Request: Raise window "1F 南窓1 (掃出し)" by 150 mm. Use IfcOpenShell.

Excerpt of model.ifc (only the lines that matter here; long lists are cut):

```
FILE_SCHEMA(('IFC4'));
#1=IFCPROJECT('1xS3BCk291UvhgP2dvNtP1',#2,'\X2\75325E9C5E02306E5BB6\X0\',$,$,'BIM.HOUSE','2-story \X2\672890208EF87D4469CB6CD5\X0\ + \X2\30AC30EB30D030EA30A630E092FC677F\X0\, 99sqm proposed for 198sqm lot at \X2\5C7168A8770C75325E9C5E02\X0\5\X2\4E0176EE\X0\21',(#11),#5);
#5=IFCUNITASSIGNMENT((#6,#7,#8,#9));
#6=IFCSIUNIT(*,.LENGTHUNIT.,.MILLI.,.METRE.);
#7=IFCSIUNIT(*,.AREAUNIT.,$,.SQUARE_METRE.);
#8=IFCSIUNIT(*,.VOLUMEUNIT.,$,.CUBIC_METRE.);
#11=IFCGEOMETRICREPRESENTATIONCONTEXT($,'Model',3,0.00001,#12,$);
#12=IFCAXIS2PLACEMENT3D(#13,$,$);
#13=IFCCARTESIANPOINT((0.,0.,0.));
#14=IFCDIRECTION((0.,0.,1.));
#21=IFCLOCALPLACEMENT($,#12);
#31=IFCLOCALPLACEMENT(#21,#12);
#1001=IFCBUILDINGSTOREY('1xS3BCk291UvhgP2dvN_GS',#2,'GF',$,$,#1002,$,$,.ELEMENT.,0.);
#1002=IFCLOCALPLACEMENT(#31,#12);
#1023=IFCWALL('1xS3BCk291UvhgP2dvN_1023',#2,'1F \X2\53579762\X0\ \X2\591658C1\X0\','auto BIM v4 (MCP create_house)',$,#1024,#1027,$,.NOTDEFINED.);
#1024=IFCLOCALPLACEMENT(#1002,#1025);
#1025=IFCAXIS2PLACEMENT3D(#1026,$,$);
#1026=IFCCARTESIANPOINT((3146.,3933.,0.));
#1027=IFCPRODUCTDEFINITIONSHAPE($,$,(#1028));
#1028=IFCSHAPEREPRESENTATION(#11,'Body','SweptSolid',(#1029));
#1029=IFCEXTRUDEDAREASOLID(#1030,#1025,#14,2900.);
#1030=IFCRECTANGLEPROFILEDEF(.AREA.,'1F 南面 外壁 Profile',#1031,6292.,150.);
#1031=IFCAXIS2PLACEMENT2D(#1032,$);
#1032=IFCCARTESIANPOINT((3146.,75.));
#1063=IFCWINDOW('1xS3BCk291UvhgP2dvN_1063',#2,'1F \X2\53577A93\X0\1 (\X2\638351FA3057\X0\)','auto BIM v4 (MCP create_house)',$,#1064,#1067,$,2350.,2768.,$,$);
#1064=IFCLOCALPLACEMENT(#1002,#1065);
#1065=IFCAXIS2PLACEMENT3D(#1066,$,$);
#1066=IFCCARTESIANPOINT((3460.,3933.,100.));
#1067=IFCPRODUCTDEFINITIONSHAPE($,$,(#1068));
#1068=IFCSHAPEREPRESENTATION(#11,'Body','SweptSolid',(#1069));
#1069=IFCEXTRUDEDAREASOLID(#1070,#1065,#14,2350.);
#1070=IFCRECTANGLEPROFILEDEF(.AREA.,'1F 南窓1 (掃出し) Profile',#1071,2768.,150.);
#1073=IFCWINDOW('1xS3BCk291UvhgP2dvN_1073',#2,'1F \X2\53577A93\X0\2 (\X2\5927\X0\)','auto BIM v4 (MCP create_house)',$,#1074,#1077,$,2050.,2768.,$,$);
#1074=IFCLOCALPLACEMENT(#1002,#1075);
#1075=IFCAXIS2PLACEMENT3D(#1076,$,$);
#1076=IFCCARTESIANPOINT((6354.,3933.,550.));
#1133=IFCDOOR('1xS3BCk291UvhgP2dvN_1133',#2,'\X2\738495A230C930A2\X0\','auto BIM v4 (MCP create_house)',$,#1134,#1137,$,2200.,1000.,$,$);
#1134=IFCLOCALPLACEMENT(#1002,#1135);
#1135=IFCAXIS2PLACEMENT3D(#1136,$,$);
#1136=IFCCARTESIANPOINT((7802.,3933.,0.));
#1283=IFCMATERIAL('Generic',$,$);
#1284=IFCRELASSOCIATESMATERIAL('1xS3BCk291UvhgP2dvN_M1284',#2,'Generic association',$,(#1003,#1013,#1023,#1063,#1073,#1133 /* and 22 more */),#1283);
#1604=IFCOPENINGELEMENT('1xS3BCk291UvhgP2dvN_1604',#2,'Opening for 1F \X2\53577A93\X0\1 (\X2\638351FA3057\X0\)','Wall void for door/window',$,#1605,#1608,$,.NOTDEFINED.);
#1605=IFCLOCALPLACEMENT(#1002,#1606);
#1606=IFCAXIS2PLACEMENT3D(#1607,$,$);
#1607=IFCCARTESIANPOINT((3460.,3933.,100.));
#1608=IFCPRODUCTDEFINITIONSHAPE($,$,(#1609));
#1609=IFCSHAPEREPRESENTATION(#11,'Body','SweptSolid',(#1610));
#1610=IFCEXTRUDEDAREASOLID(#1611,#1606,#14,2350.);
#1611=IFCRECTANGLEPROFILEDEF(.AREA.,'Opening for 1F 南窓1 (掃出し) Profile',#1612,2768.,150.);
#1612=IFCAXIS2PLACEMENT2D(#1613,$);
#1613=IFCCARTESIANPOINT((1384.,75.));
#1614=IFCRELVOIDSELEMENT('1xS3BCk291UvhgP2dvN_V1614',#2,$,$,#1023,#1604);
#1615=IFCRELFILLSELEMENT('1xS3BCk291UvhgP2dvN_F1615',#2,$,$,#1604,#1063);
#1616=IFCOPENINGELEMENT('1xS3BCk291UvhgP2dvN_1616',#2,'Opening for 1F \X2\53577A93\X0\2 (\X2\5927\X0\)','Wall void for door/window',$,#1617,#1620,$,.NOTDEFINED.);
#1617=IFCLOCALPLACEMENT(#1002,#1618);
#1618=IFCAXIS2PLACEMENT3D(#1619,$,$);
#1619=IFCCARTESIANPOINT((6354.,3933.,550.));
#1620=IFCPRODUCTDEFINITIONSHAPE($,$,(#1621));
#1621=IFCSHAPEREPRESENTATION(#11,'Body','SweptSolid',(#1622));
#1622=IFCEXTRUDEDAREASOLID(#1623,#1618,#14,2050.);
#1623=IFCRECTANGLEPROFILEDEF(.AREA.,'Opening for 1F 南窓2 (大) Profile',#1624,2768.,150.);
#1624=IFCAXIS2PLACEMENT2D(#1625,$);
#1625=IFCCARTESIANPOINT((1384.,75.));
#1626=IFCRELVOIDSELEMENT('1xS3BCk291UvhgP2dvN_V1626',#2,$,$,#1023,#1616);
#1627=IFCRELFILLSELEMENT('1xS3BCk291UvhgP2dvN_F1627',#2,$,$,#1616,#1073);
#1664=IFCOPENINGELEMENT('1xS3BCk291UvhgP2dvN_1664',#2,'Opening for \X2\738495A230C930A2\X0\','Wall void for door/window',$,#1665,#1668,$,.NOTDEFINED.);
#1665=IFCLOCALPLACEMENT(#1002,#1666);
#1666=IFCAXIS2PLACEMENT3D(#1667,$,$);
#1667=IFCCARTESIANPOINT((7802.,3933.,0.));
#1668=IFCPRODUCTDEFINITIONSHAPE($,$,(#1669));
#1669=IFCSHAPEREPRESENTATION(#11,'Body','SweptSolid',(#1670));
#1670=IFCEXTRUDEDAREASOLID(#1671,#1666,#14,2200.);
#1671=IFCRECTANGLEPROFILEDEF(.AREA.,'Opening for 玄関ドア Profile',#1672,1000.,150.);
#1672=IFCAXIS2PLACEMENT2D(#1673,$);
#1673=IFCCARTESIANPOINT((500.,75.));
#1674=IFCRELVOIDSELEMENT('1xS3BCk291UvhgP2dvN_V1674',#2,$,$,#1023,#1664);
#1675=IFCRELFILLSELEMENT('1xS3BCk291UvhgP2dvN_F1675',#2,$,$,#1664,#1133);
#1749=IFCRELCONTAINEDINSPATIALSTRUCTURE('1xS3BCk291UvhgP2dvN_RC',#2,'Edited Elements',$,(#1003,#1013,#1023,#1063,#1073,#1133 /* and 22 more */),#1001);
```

```python
import numpy as np
import ifcopenshell
import ifcopenshell.api.geometry
import ifcopenshell.util.placement
import ifcopenshell.util.unit

model = ifcopenshell.open("model.ifc")
unit_scale = ifcopenshell.util.unit.calculate_unit_scale(model)

window = model.by_id(1063)
opening = window.FillsVoids[0].RelatingOpeningElement
dz = 0.15 / unit_scale

shift = np.array([0.0, 0.0, dz])
# The window is not placed relative to its opening, so move both.
for product in (opening, window):
    matrix = ifcopenshell.util.placement.get_local_placement(product.ObjectPlacement)
    matrix[:3, 3] += shift
    ifcopenshell.api.geometry.edit_object_placement(model, product=product, matrix=matrix, is_si=False)

print(f"moved by {dz * unit_scale:+.3f} m")

model.write("model_edited.ifc")
```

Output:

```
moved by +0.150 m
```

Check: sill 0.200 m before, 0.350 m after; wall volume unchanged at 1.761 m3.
